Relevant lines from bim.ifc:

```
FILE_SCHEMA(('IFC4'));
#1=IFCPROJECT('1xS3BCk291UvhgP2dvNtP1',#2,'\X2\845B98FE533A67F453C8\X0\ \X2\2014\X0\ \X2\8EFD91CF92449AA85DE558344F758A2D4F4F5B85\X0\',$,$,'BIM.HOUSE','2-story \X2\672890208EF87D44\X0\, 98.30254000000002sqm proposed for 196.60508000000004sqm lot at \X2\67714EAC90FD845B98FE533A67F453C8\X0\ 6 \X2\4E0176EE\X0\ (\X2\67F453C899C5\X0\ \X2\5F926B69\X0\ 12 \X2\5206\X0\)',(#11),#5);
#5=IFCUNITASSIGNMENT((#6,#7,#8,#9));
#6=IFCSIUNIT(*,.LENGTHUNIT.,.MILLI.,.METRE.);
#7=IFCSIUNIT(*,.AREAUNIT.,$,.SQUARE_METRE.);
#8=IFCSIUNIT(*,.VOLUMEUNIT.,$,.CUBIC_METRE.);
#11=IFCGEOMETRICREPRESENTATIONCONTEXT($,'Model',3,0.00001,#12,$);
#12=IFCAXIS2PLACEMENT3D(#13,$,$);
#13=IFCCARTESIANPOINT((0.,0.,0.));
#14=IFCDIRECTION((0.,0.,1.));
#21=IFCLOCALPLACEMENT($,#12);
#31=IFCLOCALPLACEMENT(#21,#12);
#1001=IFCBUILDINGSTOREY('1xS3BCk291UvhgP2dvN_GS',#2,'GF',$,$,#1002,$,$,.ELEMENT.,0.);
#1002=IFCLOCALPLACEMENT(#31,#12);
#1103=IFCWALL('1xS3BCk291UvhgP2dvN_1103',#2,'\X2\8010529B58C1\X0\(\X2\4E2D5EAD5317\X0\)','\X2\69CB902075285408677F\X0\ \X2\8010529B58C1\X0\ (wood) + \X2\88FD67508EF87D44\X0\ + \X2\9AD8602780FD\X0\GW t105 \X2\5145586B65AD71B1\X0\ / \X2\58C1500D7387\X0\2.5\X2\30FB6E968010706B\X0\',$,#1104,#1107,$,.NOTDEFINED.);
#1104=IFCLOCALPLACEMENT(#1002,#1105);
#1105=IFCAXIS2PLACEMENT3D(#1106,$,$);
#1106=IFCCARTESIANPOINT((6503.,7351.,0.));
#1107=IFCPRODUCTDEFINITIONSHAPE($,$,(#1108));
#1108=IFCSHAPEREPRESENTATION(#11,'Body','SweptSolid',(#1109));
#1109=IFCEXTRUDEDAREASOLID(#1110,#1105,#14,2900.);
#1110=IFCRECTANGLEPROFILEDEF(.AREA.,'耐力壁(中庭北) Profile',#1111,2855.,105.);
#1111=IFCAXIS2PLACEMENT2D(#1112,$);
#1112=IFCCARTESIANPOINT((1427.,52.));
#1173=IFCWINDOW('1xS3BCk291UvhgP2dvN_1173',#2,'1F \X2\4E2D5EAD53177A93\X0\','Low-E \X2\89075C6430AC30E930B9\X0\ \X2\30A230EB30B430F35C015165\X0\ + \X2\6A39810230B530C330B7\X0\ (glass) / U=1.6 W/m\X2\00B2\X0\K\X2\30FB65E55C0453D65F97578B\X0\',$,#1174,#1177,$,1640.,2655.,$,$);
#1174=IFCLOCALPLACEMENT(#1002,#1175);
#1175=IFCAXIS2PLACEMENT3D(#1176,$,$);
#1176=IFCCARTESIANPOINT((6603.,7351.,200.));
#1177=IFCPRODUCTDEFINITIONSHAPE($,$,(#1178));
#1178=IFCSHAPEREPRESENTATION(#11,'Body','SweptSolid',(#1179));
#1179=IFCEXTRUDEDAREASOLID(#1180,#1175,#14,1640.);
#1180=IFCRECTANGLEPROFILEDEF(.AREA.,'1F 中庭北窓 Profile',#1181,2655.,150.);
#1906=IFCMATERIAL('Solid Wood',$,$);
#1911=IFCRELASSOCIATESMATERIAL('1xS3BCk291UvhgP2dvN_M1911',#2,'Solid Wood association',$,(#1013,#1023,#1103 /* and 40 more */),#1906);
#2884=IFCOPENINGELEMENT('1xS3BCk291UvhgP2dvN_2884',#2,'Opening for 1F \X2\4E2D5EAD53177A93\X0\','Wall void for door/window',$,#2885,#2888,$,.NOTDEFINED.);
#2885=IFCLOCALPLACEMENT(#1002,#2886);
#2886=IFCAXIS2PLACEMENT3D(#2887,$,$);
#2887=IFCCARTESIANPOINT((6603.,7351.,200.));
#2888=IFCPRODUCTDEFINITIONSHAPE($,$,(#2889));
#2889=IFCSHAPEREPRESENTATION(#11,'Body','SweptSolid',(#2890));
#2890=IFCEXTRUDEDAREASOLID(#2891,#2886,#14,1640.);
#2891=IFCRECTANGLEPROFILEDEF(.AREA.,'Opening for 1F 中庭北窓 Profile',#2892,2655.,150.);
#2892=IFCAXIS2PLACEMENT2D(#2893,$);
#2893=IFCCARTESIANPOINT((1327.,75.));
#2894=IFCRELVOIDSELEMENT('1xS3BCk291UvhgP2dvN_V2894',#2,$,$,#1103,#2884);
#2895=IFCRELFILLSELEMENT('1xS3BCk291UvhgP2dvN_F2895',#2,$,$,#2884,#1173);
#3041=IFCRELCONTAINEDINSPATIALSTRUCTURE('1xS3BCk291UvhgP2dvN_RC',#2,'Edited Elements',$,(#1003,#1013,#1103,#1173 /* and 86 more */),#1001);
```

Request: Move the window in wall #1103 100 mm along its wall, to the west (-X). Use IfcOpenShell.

```python
import ifcopenshell
import ifcopenshell.api.geometry
import ifcopenshell.util.placement
import ifcopenshell.util.unit

model = ifcopenshell.open("bim.ifc")
unit_scale = ifcopenshell.util.unit.calculate_unit_scale(model)

window = model.by_guid("1xS3BCk291UvhgP2dvN_1173")
opening = window.FillsVoids[0].RelatingOpeningElement
wall = opening.VoidsElements[0].RelatingBuildingElement

wall_matrix = ifcopenshell.util.placement.get_local_placement(wall.ObjectPlacement)
shift = wall_matrix[:3, 0] * -0.1 / unit_scale
before = ifcopenshell.util.placement.get_local_placement(window.ObjectPlacement)[:3, 3].copy()

# The window is not placed relative to its opening, so move both.
for product in (opening, window):
    matrix = ifcopenshell.util.placement.get_local_placement(product.ObjectPlacement)
    matrix[:3, 3] += shift
    ifcopenshell.api.geometry.edit_object_placement(model, product=product, matrix=matrix, is_si=False)

after = ifcopenshell.util.placement.get_local_placement(window.ObjectPlacement)[:3, 3]
print("window moved by", (after - before).round(3) + 0.0)

model.write("bim_rev.ifc")
```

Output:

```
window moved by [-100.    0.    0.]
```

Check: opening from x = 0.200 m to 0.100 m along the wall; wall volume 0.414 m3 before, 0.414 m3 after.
